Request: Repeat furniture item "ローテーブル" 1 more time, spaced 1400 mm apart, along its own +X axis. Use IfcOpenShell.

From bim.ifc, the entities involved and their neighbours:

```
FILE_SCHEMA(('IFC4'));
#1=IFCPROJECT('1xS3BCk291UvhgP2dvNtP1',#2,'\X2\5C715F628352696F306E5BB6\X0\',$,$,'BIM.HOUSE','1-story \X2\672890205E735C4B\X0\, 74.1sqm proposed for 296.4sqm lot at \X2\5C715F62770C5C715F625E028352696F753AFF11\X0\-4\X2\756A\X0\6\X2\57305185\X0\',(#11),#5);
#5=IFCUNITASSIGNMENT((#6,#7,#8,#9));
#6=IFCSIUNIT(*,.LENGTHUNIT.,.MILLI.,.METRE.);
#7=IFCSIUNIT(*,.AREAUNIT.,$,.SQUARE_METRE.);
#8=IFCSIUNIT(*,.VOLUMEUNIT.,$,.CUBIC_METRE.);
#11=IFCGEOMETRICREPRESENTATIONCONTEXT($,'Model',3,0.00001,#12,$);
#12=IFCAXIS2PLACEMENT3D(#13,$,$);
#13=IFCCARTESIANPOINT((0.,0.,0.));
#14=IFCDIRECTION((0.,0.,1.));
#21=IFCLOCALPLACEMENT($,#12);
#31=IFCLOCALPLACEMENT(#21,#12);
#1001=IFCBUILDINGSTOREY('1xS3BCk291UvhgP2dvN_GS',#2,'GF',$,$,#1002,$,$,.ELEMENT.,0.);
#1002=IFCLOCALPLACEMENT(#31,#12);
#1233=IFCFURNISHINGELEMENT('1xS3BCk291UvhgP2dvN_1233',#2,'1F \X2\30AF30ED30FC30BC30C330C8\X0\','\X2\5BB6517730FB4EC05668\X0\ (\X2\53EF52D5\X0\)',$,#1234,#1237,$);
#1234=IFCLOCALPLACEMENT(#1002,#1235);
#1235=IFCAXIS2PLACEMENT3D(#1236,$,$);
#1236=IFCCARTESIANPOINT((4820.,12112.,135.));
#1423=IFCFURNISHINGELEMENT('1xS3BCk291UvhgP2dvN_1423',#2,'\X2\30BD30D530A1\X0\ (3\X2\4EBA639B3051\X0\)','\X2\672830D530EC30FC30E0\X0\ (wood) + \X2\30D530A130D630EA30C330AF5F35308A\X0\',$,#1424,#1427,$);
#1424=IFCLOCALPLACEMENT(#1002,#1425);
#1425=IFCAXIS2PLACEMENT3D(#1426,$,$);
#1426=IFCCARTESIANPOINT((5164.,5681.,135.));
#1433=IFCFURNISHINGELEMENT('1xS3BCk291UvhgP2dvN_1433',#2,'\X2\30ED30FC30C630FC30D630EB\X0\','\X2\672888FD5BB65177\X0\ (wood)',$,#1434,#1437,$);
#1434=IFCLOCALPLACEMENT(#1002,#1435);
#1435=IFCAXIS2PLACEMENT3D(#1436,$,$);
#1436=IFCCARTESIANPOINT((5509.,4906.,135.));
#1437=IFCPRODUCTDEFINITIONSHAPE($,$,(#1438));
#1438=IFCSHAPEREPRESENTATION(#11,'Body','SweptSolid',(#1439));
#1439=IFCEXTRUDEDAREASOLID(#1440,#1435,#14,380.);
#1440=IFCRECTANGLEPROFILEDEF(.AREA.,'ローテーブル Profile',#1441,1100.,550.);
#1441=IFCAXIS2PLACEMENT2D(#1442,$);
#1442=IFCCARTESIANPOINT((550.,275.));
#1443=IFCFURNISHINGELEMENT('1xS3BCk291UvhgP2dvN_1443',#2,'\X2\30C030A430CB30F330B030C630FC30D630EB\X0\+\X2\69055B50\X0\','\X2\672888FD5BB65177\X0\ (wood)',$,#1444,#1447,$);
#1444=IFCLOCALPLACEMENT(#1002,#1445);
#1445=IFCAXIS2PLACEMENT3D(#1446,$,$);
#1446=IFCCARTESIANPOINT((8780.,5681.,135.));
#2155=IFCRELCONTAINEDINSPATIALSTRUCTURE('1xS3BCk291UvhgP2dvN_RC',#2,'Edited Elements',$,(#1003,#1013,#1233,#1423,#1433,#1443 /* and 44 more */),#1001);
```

```python
import ifcopenshell
import ifcopenshell.api.geometry
import ifcopenshell.api.root
import ifcopenshell.util.element
import ifcopenshell.util.placement
import ifcopenshell.util.unit

model = ifcopenshell.open("bim.ifc")
unit_scale = ifcopenshell.util.unit.calculate_unit_scale(model)


def reuse_history(source, copy):
    """copy_class also copies each property set's owner history, people and application; keep the originals."""
    for rel in copy.IsDefinedBy:
        if rel.is_a("IfcRelDefinesByProperties") and (history := rel.RelatingPropertyDefinition.OwnerHistory):
            rel.RelatingPropertyDefinition.OwnerHistory = source.OwnerHistory
            ifcopenshell.util.element.remove_deep2(model, history)


source = model.by_guid("1xS3BCk291UvhgP2dvN_1433")
base = ifcopenshell.util.placement.get_local_placement(source.ObjectPlacement)
step = base[:3, 0] * 1.4 / unit_scale

for i in range(1, 2):
    copy = ifcopenshell.api.root.copy_class(model, product=source)
    copy.Representation = ifcopenshell.util.element.copy_deep(
        model, source.Representation, exclude=["IfcGeometricRepresentationContext", "IfcRepresentationMap"]
    )
    reuse_history(source, copy)
    matrix = base.copy()
    matrix[:3, 3] += i * step
    print("added at", matrix[:3, 3].round(3) + 0.0)
    ifcopenshell.api.geometry.edit_object_placement(model, product=copy, matrix=matrix, is_si=False)

model.write("bim_v2.ifc")
```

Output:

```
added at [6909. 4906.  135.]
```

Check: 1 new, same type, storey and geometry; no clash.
